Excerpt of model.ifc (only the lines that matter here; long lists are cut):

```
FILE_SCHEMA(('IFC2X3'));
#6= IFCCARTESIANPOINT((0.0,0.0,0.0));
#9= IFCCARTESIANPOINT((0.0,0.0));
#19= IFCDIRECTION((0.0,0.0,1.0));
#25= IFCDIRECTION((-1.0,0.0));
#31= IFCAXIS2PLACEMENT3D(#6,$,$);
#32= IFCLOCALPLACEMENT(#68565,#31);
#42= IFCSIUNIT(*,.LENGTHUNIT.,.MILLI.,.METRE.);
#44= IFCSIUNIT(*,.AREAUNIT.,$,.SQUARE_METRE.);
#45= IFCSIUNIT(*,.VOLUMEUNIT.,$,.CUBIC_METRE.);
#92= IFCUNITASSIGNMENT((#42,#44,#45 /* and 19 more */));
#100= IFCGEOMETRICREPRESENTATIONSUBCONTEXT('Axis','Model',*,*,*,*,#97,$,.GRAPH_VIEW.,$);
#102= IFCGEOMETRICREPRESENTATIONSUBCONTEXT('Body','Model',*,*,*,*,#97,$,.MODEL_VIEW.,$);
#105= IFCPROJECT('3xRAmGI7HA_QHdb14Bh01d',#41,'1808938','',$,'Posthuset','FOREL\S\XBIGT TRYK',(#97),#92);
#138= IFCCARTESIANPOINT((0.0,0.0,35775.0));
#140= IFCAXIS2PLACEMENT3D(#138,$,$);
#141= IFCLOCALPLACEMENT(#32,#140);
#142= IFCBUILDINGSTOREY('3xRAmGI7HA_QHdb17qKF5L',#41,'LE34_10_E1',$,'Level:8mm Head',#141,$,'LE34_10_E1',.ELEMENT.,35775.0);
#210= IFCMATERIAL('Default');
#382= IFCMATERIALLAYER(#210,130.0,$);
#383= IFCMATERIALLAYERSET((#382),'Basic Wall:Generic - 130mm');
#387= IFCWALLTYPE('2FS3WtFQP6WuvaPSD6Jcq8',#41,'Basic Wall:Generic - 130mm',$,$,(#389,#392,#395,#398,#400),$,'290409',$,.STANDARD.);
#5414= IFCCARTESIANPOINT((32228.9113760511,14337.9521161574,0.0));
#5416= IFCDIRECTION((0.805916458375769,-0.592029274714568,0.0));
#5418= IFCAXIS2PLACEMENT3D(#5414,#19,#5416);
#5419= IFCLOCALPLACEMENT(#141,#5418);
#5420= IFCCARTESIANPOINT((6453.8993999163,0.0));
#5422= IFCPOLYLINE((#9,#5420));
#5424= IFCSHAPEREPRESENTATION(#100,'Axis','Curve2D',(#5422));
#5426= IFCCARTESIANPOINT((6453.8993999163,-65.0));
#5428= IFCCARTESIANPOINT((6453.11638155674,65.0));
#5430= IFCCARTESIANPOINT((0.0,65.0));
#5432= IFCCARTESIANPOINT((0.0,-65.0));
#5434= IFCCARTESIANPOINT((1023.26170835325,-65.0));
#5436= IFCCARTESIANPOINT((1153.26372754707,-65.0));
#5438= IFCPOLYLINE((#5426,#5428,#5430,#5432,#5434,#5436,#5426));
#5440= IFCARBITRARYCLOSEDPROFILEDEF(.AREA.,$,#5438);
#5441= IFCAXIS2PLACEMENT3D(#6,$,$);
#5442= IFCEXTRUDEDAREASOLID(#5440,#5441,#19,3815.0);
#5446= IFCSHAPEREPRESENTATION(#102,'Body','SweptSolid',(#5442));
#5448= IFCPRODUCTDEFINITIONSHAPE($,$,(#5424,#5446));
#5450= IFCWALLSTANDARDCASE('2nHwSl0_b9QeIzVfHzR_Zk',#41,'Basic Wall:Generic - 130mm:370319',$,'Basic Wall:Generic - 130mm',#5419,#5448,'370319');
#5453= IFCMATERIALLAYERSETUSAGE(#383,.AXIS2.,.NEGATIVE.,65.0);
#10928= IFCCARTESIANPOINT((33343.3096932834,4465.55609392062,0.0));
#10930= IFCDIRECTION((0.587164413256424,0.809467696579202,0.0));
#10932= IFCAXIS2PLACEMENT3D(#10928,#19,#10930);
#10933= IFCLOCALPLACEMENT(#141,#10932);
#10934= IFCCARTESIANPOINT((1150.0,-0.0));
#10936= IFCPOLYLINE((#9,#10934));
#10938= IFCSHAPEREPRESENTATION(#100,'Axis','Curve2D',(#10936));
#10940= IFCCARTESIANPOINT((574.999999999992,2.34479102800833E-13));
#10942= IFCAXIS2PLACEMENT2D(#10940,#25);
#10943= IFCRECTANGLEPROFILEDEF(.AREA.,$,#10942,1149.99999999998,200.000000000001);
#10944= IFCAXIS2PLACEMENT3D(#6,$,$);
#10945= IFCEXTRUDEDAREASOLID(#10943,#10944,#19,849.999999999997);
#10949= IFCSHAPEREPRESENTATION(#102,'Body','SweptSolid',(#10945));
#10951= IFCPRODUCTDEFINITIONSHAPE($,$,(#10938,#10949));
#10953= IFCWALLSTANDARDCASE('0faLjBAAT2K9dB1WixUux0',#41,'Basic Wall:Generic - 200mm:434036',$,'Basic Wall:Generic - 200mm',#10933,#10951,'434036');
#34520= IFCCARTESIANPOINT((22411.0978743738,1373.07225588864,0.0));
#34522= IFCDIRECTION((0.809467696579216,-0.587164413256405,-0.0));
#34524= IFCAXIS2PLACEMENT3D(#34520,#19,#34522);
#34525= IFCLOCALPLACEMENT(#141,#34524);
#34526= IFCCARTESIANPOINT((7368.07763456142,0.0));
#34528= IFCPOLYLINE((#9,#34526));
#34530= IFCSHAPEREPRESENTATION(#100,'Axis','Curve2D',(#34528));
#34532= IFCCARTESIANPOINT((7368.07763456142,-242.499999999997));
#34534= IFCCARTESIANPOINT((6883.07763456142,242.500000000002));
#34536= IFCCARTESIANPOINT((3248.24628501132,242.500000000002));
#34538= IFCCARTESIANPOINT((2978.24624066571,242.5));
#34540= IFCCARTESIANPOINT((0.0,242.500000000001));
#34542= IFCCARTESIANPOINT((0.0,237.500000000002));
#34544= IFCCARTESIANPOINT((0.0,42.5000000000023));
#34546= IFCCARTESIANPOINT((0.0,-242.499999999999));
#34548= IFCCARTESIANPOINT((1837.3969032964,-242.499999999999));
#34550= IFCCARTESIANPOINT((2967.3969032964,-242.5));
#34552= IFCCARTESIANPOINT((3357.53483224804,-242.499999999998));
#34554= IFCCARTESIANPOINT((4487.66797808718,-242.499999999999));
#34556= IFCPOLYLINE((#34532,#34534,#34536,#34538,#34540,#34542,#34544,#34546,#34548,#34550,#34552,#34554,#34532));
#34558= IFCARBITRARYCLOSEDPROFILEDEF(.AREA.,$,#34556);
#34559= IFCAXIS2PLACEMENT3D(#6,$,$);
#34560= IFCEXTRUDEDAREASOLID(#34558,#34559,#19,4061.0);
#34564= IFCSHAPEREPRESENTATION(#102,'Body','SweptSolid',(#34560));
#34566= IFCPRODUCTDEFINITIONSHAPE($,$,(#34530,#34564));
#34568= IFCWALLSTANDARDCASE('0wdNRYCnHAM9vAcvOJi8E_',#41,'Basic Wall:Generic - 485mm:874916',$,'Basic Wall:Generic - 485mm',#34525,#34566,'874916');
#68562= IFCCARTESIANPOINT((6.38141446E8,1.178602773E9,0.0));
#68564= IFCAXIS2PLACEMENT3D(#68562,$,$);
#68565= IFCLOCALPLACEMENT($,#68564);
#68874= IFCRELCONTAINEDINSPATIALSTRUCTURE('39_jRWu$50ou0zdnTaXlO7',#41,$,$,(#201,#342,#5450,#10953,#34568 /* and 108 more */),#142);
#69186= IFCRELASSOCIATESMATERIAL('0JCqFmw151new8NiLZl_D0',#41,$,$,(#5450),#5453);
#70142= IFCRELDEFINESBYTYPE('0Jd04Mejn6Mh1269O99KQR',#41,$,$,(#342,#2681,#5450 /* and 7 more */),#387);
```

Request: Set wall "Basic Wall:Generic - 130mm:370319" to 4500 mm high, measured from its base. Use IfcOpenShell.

```python
import ifcopenshell
import ifcopenshell.geom
import ifcopenshell.util.representation
import ifcopenshell.util.shape
import ifcopenshell.util.unit

model = ifcopenshell.open("model.ifc")
unit_scale = ifcopenshell.util.unit.calculate_unit_scale(model)
settings = ifcopenshell.geom.settings()


def volume(element):
    """Net volume in cubic metres, openings subtracted."""
    shape = ifcopenshell.geom.create_shape(settings, element)
    return ifcopenshell.util.shape.get_volume(shape.geometry)


wall = model.by_guid("2nHwSl0_b9QeIzVfHzR_Zk")
before = volume(wall)

body = ifcopenshell.util.representation.get_representation(wall, "Model", "Body")
solid = body.Items[0]
old_height = solid.Depth
solid.Depth = 4.5 / unit_scale
after = volume(wall)

print(f"height {old_height:g} -> {solid.Depth:g}, volume {before:.3f} -> {after:.3f} m3")

model.write("model_updated.ifc")
```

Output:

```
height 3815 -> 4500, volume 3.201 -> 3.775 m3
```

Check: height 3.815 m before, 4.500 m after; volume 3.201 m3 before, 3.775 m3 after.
